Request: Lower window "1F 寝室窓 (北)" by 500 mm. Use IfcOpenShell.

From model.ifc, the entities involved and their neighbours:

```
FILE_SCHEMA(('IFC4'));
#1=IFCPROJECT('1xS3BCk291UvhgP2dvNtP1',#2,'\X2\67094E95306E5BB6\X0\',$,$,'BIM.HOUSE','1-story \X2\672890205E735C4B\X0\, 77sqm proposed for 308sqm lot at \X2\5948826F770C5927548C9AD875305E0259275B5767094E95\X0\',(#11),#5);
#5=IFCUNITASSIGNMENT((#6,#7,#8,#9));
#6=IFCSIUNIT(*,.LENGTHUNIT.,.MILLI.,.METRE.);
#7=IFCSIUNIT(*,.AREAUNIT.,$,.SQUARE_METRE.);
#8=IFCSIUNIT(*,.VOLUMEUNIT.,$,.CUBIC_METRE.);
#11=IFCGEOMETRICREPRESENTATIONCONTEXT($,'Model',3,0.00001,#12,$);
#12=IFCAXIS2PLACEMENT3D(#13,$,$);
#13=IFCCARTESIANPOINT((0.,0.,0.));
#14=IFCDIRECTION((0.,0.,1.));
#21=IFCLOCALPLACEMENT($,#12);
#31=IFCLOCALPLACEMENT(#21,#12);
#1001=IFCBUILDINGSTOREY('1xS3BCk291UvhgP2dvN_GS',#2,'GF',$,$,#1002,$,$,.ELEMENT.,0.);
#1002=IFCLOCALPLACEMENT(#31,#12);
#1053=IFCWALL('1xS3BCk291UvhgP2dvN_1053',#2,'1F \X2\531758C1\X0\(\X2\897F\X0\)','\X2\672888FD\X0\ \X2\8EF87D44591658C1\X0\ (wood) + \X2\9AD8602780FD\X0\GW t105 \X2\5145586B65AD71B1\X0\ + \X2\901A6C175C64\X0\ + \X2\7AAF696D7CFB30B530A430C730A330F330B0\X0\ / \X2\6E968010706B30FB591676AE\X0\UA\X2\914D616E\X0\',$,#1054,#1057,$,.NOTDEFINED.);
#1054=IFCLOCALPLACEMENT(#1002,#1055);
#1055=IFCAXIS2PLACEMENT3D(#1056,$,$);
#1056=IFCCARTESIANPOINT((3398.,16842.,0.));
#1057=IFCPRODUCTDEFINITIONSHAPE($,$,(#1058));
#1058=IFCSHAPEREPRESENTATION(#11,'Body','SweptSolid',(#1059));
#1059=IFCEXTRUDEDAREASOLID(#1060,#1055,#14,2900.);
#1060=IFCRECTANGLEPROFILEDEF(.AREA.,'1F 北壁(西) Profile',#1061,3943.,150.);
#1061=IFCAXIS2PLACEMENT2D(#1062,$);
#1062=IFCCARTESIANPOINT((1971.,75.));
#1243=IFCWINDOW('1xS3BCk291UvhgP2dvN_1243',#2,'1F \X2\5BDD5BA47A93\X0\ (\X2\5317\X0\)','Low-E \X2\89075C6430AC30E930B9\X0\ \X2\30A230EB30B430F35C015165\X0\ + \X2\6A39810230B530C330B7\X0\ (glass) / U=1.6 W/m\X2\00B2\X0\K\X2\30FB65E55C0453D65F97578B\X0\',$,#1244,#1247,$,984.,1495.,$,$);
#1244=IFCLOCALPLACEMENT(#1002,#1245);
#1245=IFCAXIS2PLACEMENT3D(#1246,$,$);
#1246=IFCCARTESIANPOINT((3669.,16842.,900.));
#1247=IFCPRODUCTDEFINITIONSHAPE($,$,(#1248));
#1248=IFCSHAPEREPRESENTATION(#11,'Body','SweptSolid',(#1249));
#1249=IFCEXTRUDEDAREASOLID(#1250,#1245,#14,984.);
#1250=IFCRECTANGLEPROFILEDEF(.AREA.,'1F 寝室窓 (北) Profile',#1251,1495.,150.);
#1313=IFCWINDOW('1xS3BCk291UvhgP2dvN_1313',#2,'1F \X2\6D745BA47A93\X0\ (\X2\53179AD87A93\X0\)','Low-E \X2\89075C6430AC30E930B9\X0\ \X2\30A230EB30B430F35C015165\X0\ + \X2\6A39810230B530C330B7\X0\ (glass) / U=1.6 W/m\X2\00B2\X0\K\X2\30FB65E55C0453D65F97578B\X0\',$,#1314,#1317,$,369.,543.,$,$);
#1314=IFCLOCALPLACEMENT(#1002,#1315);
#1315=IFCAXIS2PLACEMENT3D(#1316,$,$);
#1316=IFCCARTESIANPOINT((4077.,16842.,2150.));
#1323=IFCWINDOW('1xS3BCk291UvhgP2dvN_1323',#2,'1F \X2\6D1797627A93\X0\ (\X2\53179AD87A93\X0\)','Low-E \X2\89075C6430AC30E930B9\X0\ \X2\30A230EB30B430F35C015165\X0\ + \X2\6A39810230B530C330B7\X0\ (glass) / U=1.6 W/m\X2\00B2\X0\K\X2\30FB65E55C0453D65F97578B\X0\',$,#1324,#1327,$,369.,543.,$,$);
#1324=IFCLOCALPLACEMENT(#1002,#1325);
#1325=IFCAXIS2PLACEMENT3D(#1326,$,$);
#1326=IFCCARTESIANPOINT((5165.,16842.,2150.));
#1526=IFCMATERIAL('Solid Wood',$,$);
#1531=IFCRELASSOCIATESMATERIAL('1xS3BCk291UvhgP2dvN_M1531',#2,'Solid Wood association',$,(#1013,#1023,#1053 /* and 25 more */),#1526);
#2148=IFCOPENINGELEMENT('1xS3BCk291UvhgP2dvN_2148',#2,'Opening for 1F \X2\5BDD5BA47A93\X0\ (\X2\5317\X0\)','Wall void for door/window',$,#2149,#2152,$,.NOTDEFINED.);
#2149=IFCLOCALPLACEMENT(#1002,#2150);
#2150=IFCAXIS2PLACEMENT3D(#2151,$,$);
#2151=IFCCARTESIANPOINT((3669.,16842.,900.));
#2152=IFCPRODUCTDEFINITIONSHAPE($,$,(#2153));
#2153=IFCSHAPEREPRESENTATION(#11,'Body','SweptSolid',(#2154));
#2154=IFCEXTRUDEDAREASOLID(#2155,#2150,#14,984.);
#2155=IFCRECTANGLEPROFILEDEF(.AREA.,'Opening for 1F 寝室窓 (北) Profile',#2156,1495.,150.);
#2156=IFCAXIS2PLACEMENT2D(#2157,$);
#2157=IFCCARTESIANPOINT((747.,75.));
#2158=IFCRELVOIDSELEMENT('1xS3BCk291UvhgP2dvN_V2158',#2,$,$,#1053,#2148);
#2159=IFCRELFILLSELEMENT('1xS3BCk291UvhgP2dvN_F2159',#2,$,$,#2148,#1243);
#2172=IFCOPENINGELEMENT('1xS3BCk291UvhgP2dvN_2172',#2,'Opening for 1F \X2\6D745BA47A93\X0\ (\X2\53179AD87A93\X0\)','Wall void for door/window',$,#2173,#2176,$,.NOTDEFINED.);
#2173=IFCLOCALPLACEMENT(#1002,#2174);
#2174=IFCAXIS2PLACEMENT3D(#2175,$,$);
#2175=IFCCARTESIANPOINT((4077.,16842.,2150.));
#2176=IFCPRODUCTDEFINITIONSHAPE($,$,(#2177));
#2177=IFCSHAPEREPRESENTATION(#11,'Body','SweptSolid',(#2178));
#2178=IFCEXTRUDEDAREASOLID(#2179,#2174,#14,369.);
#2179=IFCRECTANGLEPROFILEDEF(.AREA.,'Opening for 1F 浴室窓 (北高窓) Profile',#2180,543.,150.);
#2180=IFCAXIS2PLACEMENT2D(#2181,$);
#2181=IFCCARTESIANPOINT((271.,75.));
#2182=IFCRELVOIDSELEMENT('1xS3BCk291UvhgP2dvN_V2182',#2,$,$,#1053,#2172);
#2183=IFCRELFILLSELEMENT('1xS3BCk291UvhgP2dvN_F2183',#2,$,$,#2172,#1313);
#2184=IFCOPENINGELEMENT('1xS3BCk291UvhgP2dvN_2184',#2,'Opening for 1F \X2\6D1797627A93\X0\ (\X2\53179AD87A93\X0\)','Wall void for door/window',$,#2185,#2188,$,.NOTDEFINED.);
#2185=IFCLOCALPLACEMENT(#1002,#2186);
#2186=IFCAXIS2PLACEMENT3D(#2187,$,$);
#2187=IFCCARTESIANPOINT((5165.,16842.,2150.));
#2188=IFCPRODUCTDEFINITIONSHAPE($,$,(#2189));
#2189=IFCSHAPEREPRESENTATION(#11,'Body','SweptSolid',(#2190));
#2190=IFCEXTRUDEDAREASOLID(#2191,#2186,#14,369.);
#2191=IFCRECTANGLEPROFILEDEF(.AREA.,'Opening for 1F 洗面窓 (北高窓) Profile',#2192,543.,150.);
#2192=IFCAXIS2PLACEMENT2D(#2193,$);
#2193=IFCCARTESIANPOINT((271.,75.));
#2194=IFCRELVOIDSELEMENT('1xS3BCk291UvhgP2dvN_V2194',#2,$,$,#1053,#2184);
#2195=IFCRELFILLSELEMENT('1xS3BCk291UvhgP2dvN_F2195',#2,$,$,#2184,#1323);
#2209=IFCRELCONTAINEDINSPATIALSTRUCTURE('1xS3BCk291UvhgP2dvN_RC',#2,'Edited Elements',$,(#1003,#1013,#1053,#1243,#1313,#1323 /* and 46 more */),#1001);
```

```python
import numpy as np
import ifcopenshell
import ifcopenshell.api.geometry
import ifcopenshell.util.placement
import ifcopenshell.util.unit

model = ifcopenshell.open("model.ifc")
unit_scale = ifcopenshell.util.unit.calculate_unit_scale(model)

window = model.by_guid("1xS3BCk291UvhgP2dvN_1243")
opening = window.FillsVoids[0].RelatingOpeningElement
dz = -500.0

shift = np.array([0.0, 0.0, dz])
# The window is not placed relative to its opening, so move both.
for product in (opening, window):
    matrix = ifcopenshell.util.placement.get_local_placement(product.ObjectPlacement)
    matrix[:3, 3] += shift
    ifcopenshell.api.geometry.edit_object_placement(model, product=product, matrix=matrix, is_si=False)

print(f"moved by {dz * unit_scale:+.3f} m")

model.write("model_rev.ifc")
```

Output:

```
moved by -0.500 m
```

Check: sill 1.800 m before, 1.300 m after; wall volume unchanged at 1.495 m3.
